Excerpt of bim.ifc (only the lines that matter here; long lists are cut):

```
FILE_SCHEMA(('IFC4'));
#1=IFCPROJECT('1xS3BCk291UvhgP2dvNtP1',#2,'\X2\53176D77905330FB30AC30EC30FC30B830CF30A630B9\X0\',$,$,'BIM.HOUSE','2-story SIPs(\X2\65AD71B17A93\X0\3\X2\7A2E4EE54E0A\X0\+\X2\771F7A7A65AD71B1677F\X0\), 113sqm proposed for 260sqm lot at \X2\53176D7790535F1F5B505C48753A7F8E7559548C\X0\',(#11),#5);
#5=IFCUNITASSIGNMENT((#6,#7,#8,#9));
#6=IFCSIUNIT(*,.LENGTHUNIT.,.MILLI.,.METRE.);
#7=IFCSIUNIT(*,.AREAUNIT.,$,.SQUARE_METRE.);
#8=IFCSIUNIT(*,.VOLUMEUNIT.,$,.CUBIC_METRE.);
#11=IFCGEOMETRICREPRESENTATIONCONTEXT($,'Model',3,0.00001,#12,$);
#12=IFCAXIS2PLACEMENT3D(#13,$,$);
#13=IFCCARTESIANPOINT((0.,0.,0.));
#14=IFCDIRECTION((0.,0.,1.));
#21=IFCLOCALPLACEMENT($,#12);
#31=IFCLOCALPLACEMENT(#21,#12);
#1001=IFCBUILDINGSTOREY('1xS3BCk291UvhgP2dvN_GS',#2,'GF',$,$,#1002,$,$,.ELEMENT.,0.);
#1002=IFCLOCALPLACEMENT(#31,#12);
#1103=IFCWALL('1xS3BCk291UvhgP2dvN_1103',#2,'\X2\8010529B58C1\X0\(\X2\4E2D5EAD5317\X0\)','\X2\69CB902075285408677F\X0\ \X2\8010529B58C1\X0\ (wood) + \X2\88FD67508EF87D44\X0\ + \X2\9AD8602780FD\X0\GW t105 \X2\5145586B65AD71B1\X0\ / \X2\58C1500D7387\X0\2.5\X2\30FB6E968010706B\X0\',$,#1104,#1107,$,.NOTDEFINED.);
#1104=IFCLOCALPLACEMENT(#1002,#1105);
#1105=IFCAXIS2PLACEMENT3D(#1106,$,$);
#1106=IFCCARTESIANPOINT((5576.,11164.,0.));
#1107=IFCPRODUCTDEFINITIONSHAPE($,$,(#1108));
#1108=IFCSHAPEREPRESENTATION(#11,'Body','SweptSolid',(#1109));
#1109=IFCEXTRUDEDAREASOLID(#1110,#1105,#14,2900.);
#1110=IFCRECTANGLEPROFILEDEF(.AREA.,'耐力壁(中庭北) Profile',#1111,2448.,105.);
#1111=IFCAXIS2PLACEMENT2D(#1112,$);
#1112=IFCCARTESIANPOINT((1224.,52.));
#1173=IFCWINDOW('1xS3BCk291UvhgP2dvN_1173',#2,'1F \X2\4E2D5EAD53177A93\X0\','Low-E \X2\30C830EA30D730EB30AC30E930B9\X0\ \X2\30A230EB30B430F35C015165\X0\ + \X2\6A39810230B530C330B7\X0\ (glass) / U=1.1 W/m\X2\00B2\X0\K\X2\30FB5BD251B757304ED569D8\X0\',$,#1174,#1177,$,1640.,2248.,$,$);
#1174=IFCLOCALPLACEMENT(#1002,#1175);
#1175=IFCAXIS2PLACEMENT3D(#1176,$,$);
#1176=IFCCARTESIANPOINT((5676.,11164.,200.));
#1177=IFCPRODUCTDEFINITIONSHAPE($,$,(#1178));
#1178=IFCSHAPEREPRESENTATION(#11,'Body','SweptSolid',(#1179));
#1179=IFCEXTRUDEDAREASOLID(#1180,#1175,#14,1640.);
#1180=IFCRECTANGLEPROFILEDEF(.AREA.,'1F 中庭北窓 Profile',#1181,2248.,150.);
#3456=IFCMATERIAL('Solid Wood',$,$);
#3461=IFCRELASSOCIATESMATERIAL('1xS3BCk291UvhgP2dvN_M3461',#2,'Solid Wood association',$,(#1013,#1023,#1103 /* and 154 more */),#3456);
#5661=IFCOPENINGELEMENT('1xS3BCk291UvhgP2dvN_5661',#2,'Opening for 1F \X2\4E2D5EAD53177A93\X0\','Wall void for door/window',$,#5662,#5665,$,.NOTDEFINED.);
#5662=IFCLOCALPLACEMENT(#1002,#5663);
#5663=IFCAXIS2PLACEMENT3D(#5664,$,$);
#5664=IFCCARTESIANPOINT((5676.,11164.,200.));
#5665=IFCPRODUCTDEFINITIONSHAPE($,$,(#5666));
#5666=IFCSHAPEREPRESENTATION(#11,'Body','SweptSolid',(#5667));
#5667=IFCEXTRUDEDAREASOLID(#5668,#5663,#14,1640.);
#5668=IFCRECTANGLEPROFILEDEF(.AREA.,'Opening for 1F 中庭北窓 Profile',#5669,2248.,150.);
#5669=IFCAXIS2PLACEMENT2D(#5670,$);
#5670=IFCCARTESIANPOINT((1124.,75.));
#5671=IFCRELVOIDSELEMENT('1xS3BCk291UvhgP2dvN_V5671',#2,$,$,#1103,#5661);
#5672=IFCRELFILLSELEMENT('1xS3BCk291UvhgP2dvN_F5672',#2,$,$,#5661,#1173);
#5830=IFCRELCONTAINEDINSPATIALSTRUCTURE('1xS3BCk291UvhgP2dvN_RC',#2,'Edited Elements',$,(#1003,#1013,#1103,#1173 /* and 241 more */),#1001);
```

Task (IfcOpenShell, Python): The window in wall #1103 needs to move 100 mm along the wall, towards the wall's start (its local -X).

```python
import ifcopenshell
import ifcopenshell.api.geometry
import ifcopenshell.util.placement
import ifcopenshell.util.unit

model = ifcopenshell.open("bim.ifc")
unit_scale = ifcopenshell.util.unit.calculate_unit_scale(model)

window = model.by_id(1173)
opening = window.FillsVoids[0].RelatingOpeningElement
wall = opening.VoidsElements[0].RelatingBuildingElement

wall_matrix = ifcopenshell.util.placement.get_local_placement(wall.ObjectPlacement)
shift = wall_matrix[:3, 0] * -0.1 / unit_scale
before = ifcopenshell.util.placement.get_local_placement(window.ObjectPlacement)[:3, 3].copy()

# The window is not placed relative to its opening, so move both.
for product in (opening, window):
    matrix = ifcopenshell.util.placement.get_local_placement(product.ObjectPlacement)
    matrix[:3, 3] += shift
    ifcopenshell.api.geometry.edit_object_placement(model, product=product, matrix=matrix, is_si=False)

after = ifcopenshell.util.placement.get_local_placement(window.ObjectPlacement)[:3, 3]
print("window moved by", (after - before).round(3) + 0.0)

model.write("bim_rev.ifc")
```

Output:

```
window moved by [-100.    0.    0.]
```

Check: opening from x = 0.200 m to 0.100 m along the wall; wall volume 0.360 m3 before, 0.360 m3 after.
